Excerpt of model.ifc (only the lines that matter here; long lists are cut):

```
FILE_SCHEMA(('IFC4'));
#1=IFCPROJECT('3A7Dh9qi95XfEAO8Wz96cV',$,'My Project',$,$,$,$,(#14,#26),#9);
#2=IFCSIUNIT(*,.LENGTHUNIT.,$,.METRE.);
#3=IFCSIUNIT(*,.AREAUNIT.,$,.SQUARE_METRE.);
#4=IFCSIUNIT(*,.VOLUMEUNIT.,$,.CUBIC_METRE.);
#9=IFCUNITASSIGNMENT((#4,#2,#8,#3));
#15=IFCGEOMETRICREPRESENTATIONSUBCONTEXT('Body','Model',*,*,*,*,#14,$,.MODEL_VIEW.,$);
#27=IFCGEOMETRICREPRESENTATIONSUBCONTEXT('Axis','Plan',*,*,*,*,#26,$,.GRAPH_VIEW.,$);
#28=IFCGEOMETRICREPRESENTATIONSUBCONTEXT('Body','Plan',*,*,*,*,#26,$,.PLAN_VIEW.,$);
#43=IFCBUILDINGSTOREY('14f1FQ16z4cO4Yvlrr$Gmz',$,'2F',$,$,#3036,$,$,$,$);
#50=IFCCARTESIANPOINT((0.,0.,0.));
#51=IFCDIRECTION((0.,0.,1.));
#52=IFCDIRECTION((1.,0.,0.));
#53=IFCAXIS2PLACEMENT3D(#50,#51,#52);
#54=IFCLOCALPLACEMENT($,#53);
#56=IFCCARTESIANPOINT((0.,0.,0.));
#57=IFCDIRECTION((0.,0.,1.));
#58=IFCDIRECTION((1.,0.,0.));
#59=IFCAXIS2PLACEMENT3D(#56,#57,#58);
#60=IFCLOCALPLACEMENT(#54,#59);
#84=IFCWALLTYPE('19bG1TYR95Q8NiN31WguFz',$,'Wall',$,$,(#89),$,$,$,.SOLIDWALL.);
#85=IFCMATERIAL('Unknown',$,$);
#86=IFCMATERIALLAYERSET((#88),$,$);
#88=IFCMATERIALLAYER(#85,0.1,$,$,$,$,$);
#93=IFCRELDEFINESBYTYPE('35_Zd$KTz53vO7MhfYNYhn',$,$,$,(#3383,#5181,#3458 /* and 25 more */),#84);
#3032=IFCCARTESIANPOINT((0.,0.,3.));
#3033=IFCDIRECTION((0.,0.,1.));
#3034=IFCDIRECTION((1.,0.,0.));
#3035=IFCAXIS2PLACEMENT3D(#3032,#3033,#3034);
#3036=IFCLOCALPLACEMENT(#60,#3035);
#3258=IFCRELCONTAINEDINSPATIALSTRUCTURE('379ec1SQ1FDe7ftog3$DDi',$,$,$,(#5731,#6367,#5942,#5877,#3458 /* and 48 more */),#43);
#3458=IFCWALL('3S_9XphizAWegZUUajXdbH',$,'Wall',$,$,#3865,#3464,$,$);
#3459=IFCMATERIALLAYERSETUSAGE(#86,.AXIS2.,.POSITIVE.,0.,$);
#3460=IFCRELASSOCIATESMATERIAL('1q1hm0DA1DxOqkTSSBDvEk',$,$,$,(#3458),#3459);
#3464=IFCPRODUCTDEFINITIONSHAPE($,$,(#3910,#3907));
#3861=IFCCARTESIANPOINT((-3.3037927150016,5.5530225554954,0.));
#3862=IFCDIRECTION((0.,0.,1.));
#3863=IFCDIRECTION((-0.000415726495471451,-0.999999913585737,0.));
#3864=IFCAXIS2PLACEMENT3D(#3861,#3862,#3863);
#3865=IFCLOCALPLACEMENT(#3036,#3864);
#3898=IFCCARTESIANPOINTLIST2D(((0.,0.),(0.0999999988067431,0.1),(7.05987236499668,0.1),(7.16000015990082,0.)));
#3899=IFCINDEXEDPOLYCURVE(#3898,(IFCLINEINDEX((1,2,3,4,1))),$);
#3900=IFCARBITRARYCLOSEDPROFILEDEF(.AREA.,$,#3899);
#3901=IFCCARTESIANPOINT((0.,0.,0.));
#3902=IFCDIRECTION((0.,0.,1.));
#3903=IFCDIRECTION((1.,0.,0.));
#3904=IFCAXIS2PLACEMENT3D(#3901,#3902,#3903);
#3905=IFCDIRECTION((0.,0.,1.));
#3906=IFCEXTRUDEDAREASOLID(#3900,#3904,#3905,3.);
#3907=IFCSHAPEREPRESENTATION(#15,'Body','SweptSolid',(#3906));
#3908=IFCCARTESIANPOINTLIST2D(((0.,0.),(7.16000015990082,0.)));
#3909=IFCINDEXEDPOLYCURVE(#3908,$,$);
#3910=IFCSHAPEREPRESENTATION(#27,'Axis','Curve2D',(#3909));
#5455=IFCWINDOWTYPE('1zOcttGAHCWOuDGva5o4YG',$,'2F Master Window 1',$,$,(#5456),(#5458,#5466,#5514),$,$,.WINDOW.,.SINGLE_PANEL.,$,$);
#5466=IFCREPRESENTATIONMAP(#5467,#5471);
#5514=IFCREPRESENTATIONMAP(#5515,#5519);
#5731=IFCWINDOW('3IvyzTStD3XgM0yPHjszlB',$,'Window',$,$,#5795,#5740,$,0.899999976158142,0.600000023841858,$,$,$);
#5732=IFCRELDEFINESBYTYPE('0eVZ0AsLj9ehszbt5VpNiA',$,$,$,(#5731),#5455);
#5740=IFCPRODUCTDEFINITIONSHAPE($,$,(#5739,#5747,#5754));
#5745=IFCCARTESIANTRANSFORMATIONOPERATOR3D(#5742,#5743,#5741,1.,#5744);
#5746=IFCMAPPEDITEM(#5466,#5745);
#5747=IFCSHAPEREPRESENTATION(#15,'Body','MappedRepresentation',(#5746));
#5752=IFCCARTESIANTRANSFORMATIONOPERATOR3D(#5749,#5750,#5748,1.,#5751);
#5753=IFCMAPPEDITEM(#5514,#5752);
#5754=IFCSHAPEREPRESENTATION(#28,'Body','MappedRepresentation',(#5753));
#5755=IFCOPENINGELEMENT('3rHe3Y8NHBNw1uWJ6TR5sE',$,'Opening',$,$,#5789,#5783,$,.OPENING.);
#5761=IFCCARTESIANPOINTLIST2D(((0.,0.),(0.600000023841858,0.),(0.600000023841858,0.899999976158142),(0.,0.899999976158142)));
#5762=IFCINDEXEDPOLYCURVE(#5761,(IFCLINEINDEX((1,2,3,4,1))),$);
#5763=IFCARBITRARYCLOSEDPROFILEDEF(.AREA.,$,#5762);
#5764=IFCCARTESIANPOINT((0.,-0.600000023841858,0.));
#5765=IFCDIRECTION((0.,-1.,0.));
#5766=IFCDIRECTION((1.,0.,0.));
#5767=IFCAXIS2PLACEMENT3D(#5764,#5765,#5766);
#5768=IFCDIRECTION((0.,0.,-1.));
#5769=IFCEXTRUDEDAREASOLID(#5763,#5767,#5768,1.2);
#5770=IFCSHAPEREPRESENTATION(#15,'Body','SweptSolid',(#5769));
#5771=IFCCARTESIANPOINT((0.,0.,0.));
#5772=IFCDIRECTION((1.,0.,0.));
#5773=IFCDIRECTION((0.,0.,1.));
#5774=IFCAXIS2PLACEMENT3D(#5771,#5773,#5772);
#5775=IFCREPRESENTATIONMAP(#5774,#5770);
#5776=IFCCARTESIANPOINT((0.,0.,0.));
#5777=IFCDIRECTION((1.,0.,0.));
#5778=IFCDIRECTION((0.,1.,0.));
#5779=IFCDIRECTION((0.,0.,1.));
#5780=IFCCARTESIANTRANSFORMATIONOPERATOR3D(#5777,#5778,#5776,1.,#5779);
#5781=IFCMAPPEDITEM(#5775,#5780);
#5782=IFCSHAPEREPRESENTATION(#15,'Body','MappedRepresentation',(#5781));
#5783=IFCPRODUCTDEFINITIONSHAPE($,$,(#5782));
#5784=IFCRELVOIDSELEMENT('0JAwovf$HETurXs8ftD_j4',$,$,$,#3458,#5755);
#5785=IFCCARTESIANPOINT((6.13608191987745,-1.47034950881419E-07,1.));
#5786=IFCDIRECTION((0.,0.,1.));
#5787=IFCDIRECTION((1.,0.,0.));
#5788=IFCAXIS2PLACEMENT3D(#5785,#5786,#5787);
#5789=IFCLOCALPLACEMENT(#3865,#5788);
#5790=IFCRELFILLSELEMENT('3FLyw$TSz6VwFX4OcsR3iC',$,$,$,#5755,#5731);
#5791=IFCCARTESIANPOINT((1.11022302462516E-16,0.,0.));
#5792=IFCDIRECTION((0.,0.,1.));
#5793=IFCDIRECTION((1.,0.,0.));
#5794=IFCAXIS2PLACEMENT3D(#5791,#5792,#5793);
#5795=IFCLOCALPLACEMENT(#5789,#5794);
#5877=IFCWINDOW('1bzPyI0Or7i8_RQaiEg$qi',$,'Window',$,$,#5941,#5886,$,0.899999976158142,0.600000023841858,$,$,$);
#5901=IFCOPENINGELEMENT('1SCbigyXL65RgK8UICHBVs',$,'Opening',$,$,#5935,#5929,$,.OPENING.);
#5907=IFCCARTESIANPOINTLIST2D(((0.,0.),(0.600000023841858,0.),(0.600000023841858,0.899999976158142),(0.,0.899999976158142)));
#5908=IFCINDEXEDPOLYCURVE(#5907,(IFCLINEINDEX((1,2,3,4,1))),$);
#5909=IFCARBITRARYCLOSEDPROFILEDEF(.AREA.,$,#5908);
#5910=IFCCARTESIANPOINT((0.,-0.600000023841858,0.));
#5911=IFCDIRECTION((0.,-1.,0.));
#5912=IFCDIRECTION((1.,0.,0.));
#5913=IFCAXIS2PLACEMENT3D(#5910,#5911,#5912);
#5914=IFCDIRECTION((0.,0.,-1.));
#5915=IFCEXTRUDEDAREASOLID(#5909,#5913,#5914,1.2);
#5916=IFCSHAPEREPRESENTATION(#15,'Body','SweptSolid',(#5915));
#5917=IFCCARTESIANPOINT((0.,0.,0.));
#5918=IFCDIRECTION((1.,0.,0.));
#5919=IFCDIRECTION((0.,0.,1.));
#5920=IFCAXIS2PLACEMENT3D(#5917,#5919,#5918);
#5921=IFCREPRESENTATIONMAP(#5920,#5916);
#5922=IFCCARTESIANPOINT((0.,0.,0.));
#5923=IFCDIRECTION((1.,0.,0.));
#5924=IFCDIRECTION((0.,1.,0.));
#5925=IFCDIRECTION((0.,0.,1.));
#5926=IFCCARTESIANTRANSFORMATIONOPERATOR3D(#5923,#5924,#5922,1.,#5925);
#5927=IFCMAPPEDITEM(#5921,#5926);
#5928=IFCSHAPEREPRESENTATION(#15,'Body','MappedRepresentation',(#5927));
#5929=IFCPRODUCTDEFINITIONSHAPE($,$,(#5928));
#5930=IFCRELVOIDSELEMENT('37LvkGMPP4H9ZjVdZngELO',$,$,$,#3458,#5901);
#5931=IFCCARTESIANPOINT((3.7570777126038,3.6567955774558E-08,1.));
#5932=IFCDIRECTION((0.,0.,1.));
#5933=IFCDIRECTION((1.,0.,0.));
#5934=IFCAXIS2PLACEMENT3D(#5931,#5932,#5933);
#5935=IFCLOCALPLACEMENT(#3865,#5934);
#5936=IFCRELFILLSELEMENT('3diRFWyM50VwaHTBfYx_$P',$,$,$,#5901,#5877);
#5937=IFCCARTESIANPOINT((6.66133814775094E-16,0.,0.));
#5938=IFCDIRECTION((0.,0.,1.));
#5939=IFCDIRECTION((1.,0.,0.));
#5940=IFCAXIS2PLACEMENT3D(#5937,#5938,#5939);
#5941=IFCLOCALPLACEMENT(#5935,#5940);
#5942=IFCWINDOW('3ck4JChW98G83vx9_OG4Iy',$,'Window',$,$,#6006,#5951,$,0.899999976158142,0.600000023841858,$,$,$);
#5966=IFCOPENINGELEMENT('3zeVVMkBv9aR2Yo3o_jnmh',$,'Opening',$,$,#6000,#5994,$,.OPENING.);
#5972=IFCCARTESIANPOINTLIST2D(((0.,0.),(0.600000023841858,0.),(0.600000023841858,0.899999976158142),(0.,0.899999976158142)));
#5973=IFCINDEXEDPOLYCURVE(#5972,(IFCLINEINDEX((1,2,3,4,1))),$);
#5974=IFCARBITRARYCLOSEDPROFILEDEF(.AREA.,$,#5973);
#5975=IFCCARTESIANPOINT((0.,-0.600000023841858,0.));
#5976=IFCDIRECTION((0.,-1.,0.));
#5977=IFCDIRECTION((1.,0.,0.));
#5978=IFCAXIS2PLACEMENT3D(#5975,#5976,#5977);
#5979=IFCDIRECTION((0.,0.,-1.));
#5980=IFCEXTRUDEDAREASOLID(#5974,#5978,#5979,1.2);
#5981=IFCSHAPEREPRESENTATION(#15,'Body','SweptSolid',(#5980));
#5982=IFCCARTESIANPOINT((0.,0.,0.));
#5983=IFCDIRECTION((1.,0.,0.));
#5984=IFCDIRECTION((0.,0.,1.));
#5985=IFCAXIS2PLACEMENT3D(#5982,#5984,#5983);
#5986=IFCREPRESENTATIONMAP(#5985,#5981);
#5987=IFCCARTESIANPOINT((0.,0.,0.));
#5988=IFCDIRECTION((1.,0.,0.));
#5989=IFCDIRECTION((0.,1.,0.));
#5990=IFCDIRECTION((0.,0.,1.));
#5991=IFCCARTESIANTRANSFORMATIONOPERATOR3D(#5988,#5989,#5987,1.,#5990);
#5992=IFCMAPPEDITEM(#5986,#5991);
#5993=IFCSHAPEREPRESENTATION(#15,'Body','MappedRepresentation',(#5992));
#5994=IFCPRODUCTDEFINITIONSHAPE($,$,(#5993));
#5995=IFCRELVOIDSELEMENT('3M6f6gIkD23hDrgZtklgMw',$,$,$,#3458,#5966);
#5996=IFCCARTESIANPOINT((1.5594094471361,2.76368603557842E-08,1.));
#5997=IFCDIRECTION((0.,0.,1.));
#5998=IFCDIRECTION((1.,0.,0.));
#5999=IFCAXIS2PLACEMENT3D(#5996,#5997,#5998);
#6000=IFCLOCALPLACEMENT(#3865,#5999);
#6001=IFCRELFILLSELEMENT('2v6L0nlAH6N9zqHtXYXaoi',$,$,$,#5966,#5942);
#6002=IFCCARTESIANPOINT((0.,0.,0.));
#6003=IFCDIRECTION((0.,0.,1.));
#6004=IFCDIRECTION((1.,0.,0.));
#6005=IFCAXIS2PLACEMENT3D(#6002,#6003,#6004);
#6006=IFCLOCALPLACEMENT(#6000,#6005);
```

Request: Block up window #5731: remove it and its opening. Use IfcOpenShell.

```python
import ifcopenshell
import ifcopenshell.api.feature
import ifcopenshell.api.root
import ifcopenshell.geom
import ifcopenshell.util.shape

model = ifcopenshell.open("model.ifc")
settings = ifcopenshell.geom.settings()


def volume(element):
    """Net volume in cubic metres, openings subtracted."""
    shape = ifcopenshell.geom.create_shape(settings, element)
    return ifcopenshell.util.shape.get_volume(shape.geometry)


window = model.by_id(5731)
opening = window.FillsVoids[0].RelatingOpeningElement
wall = opening.VoidsElements[0].RelatingBuildingElement
before = volume(wall)

ifcopenshell.api.root.remove_product(model, product=window)
ifcopenshell.api.feature.remove_feature(model, feature=opening)

after = volume(wall)

print(f"wall volume {before:.3f} -> {after:.3f} m3")

model.write("model_v2.ifc")
```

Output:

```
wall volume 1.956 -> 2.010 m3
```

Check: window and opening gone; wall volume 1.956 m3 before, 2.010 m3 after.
